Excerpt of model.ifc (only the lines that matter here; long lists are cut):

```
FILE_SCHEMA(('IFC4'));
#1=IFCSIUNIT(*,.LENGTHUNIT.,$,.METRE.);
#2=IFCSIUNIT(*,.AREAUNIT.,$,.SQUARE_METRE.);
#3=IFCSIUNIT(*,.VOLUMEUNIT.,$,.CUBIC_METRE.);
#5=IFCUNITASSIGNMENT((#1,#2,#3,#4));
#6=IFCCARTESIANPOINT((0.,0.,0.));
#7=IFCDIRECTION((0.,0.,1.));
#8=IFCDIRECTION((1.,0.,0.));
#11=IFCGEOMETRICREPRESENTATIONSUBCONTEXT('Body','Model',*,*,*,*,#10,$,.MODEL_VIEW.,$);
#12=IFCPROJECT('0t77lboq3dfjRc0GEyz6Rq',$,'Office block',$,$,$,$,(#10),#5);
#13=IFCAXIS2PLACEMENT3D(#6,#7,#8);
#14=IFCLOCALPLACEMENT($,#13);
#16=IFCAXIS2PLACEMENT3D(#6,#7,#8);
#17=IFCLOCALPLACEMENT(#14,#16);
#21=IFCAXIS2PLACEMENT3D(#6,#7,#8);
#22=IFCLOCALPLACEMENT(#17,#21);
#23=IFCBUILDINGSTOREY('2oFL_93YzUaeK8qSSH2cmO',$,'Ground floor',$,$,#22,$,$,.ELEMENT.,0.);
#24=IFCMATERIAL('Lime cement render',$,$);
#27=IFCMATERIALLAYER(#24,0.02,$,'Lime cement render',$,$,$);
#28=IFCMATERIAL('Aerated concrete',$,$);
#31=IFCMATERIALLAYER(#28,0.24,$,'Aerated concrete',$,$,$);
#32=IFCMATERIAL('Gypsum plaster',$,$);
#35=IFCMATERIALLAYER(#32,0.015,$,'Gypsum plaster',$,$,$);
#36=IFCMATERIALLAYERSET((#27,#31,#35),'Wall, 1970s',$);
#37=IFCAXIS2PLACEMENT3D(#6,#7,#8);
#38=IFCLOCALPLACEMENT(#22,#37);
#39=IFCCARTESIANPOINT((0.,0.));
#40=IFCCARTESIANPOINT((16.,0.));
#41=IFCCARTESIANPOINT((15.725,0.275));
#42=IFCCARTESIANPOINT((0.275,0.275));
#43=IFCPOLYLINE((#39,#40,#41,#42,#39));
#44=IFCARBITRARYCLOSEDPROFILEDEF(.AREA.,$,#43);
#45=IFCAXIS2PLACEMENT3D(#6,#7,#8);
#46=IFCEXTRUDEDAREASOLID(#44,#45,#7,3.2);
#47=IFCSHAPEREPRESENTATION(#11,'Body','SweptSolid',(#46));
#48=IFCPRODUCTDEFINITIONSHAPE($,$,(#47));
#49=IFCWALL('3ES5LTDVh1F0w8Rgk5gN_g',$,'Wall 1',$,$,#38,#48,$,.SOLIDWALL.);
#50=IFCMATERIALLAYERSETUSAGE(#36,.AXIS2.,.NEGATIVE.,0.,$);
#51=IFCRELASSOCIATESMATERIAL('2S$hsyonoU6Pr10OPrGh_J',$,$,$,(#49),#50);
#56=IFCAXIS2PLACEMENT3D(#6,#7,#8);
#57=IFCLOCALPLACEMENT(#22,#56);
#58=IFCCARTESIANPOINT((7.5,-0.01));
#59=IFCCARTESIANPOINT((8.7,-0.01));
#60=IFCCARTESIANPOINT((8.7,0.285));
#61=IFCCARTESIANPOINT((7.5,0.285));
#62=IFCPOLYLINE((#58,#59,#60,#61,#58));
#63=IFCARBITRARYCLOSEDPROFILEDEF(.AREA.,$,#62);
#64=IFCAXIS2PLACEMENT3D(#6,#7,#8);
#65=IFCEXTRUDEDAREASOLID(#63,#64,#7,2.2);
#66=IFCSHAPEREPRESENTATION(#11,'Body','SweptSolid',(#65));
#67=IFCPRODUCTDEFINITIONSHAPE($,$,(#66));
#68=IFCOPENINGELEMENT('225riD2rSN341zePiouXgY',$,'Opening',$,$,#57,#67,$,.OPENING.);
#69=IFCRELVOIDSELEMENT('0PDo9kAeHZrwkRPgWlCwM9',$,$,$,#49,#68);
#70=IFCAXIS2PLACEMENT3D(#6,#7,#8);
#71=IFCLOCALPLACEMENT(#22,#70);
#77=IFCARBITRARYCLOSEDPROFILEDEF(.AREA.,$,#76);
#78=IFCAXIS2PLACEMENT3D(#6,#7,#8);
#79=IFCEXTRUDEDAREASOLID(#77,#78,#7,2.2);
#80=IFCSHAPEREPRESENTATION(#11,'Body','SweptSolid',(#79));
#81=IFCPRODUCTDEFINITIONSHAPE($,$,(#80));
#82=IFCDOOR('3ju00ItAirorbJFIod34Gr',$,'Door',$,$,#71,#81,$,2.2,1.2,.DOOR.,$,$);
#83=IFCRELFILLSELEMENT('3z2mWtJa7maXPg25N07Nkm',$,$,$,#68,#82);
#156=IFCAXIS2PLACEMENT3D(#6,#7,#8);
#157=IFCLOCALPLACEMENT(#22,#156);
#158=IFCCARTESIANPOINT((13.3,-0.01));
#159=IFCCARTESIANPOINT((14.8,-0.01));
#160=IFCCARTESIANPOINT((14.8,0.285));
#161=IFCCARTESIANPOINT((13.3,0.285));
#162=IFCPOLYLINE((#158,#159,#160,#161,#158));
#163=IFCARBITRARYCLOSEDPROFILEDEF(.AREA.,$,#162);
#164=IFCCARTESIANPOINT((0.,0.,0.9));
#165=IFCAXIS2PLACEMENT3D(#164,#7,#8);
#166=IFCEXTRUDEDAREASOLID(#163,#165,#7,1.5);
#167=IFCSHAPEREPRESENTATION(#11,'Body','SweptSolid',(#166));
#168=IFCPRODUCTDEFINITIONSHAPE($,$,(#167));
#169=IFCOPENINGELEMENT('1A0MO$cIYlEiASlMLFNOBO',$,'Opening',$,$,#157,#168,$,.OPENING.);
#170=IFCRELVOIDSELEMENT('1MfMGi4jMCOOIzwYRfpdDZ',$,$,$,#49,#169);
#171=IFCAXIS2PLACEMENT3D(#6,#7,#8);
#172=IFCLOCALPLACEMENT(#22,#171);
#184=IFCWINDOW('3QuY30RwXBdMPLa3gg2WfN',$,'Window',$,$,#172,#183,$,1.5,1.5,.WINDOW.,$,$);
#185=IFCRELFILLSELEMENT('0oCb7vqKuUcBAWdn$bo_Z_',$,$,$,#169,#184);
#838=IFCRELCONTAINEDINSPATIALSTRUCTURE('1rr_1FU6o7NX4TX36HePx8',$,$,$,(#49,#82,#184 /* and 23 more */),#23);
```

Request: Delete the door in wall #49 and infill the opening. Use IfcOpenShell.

```python
import ifcopenshell
import ifcopenshell.api.feature
import ifcopenshell.api.root
import ifcopenshell.geom
import ifcopenshell.util.shape

model = ifcopenshell.open("model.ifc")
settings = ifcopenshell.geom.settings()


def volume(element):
    """Net volume in cubic metres, openings subtracted."""
    shape = ifcopenshell.geom.create_shape(settings, element)
    return ifcopenshell.util.shape.get_volume(shape.geometry)


door = model.by_guid("3ju00ItAirorbJFIod34Gr")
opening = door.FillsVoids[0].RelatingOpeningElement
wall = opening.VoidsElements[0].RelatingBuildingElement
before = volume(wall)

ifcopenshell.api.root.remove_product(model, product=door)
ifcopenshell.api.feature.remove_feature(model, feature=opening)

after = volume(wall)

print(f"wall volume {before:.3f} -> {after:.3f} m3")

model.write("model_updated.ifc")
```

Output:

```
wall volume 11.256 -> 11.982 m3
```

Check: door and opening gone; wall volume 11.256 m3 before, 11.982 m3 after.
